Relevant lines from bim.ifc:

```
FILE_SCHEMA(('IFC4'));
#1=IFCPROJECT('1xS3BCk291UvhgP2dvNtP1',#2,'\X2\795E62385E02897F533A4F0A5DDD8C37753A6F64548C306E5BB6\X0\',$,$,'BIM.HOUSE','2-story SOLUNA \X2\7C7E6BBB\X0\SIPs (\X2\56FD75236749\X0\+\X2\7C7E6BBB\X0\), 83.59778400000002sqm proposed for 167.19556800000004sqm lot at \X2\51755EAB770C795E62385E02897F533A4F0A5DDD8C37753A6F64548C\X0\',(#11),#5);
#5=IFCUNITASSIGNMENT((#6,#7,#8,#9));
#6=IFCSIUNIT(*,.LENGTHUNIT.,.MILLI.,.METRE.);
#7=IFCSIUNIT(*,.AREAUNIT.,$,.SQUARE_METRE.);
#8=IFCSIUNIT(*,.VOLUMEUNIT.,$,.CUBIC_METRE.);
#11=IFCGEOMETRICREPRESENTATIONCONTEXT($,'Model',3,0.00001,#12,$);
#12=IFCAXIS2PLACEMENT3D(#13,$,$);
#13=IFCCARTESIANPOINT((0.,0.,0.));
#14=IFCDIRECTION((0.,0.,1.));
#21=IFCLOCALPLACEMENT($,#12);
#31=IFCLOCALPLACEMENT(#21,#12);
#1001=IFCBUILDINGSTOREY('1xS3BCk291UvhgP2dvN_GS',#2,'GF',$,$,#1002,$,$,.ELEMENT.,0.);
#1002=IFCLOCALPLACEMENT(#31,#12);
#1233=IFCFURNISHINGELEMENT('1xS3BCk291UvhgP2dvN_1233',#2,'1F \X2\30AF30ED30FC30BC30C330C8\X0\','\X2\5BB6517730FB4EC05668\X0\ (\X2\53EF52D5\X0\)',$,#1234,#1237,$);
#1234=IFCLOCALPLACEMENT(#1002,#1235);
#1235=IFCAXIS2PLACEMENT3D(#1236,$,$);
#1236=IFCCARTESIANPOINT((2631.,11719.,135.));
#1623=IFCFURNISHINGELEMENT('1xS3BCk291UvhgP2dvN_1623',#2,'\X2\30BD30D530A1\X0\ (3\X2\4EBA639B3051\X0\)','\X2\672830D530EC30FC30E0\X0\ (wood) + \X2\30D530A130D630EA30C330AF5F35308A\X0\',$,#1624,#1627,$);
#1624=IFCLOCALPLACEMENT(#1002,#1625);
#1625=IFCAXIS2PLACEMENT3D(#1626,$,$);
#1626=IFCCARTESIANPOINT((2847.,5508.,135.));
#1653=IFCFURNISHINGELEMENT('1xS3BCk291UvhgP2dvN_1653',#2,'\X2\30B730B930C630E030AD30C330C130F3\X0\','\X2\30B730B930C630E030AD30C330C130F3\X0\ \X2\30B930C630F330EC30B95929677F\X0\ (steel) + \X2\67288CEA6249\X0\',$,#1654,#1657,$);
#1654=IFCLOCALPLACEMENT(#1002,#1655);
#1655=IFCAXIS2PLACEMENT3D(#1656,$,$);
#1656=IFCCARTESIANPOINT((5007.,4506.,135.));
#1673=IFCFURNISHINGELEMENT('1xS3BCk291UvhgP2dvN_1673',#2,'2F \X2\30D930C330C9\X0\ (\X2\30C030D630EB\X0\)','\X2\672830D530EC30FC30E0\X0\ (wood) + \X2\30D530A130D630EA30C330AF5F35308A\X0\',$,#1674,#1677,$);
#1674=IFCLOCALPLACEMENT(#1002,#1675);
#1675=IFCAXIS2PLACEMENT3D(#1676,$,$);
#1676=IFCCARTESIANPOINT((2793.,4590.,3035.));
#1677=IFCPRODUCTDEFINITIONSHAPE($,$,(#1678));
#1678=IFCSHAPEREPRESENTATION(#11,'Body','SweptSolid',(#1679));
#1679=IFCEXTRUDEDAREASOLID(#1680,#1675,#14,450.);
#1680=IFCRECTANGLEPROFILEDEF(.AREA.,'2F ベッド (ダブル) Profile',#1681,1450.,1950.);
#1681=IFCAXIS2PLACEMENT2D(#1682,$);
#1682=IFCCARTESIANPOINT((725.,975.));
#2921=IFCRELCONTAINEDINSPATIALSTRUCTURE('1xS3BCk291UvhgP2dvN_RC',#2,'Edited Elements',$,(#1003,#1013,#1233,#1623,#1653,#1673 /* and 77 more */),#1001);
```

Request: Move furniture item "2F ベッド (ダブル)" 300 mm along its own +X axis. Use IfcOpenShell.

```python
import ifcopenshell
import ifcopenshell.api.geometry
import ifcopenshell.util.placement
import ifcopenshell.util.unit

model = ifcopenshell.open("bim.ifc")
unit_scale = ifcopenshell.util.unit.calculate_unit_scale(model)

item = model.by_guid("1xS3BCk291UvhgP2dvN_1673")
matrix = ifcopenshell.util.placement.get_local_placement(item.ObjectPlacement)
matrix[:3, 3] += matrix[:3, 0] * 0.3 / unit_scale
ifcopenshell.api.geometry.edit_object_placement(model, product=item, matrix=matrix, is_si=False)

print(ifcopenshell.util.placement.get_local_placement(item.ObjectPlacement).round(3) + 0.0)

model.write("bim-out.ifc")
```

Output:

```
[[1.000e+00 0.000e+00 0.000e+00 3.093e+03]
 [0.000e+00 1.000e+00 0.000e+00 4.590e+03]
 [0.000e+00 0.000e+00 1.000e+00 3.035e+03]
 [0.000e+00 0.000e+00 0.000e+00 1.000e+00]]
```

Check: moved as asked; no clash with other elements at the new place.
